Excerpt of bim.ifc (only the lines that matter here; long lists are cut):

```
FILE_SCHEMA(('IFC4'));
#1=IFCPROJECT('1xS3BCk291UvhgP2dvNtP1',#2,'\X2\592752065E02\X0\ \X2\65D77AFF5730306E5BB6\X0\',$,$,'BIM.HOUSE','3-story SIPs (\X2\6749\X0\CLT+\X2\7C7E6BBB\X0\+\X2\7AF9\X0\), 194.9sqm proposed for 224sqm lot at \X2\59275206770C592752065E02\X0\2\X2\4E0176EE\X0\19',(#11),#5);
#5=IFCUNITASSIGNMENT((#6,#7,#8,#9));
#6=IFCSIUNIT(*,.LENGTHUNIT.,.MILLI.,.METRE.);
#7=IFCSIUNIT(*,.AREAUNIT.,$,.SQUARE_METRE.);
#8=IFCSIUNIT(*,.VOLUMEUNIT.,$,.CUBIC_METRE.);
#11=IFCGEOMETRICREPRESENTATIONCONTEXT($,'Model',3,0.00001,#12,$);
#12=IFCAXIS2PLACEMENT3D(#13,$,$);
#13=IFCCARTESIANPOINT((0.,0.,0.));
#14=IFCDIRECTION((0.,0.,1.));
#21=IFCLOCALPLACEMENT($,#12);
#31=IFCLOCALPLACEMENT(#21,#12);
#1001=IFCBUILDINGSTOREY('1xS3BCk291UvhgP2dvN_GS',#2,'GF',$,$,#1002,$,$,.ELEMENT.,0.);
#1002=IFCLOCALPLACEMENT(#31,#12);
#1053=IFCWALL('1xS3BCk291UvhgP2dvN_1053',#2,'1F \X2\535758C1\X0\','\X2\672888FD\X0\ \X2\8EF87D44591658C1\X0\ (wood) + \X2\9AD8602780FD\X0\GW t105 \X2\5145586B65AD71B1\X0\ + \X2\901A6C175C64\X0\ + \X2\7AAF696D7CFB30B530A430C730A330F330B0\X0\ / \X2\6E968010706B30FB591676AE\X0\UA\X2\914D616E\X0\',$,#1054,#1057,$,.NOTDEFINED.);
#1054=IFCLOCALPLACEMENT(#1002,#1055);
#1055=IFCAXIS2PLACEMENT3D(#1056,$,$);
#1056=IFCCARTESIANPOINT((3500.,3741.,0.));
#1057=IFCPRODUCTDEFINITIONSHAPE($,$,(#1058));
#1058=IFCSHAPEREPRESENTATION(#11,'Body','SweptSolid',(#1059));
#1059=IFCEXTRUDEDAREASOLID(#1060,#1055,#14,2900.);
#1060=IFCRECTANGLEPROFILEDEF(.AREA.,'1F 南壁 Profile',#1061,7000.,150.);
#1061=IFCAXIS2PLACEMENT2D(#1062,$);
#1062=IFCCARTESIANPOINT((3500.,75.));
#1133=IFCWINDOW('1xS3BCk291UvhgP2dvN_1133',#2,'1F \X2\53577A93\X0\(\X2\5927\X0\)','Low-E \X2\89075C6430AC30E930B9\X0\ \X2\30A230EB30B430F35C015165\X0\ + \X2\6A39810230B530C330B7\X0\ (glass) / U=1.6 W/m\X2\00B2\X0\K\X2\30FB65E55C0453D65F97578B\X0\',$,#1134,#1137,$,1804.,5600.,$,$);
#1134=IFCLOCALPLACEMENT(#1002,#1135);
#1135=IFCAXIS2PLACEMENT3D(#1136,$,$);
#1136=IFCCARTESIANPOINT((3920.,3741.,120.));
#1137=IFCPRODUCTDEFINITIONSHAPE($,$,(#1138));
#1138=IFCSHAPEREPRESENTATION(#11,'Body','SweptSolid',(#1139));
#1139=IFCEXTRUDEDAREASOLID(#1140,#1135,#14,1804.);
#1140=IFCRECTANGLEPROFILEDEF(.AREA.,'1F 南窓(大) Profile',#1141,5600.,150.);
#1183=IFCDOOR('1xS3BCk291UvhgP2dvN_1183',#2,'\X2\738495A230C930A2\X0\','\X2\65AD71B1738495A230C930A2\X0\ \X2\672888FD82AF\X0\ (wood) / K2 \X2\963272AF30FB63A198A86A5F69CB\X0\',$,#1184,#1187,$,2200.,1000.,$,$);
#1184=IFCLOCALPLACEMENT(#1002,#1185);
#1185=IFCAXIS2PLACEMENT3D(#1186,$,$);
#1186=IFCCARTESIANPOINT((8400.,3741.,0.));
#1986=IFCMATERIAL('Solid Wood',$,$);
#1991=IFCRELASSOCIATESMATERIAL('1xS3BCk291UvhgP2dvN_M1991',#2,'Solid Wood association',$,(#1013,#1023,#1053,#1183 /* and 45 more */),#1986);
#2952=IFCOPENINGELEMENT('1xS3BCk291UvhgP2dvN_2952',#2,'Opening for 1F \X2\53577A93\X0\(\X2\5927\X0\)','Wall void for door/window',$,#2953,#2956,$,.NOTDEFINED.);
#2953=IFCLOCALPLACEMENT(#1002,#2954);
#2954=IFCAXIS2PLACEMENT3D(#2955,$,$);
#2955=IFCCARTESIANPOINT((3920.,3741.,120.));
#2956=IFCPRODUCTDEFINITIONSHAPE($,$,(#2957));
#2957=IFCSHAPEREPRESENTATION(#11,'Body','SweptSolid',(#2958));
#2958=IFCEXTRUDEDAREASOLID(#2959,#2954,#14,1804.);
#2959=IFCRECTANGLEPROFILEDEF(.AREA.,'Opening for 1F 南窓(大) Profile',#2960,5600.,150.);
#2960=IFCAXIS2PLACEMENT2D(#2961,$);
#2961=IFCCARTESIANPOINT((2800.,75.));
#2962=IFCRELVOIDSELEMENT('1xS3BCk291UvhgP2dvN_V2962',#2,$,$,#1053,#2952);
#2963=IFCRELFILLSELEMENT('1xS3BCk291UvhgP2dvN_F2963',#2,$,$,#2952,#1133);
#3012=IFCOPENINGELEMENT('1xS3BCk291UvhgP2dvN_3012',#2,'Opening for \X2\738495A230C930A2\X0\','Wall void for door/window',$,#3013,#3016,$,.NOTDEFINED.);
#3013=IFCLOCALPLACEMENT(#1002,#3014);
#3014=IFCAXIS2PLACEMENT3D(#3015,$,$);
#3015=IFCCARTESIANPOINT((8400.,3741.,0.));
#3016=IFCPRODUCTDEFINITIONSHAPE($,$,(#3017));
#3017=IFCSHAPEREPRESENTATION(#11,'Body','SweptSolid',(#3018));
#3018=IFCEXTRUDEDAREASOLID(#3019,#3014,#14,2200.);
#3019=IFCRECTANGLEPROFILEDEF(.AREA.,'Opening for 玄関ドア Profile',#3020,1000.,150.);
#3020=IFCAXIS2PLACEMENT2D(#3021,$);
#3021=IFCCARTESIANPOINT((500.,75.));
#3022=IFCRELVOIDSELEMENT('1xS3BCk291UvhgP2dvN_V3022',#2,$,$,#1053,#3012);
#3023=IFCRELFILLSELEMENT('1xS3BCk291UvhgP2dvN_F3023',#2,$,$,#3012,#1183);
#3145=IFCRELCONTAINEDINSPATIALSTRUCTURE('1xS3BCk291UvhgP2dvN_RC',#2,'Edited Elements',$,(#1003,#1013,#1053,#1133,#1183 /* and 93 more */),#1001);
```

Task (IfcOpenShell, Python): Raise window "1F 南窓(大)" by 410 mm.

```python
import numpy as np
import ifcopenshell
import ifcopenshell.api.geometry
import ifcopenshell.util.placement
import ifcopenshell.util.unit

model = ifcopenshell.open("bim.ifc")
unit_scale = ifcopenshell.util.unit.calculate_unit_scale(model)

window = model.by_guid("1xS3BCk291UvhgP2dvN_1133")
opening = window.FillsVoids[0].RelatingOpeningElement
dz = 410.0

shift = np.array([0.0, 0.0, dz])
# The window is not placed relative to its opening, so move both.
for product in (opening, window):
    matrix = ifcopenshell.util.placement.get_local_placement(product.ObjectPlacement)
    matrix[:3, 3] += shift
    ifcopenshell.api.geometry.edit_object_placement(model, product=product, matrix=matrix, is_si=False)

print(f"moved by {dz * unit_scale:+.3f} m")

model.write("bim_edited.ifc")
```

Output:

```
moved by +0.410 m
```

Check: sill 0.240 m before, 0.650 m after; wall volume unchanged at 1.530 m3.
